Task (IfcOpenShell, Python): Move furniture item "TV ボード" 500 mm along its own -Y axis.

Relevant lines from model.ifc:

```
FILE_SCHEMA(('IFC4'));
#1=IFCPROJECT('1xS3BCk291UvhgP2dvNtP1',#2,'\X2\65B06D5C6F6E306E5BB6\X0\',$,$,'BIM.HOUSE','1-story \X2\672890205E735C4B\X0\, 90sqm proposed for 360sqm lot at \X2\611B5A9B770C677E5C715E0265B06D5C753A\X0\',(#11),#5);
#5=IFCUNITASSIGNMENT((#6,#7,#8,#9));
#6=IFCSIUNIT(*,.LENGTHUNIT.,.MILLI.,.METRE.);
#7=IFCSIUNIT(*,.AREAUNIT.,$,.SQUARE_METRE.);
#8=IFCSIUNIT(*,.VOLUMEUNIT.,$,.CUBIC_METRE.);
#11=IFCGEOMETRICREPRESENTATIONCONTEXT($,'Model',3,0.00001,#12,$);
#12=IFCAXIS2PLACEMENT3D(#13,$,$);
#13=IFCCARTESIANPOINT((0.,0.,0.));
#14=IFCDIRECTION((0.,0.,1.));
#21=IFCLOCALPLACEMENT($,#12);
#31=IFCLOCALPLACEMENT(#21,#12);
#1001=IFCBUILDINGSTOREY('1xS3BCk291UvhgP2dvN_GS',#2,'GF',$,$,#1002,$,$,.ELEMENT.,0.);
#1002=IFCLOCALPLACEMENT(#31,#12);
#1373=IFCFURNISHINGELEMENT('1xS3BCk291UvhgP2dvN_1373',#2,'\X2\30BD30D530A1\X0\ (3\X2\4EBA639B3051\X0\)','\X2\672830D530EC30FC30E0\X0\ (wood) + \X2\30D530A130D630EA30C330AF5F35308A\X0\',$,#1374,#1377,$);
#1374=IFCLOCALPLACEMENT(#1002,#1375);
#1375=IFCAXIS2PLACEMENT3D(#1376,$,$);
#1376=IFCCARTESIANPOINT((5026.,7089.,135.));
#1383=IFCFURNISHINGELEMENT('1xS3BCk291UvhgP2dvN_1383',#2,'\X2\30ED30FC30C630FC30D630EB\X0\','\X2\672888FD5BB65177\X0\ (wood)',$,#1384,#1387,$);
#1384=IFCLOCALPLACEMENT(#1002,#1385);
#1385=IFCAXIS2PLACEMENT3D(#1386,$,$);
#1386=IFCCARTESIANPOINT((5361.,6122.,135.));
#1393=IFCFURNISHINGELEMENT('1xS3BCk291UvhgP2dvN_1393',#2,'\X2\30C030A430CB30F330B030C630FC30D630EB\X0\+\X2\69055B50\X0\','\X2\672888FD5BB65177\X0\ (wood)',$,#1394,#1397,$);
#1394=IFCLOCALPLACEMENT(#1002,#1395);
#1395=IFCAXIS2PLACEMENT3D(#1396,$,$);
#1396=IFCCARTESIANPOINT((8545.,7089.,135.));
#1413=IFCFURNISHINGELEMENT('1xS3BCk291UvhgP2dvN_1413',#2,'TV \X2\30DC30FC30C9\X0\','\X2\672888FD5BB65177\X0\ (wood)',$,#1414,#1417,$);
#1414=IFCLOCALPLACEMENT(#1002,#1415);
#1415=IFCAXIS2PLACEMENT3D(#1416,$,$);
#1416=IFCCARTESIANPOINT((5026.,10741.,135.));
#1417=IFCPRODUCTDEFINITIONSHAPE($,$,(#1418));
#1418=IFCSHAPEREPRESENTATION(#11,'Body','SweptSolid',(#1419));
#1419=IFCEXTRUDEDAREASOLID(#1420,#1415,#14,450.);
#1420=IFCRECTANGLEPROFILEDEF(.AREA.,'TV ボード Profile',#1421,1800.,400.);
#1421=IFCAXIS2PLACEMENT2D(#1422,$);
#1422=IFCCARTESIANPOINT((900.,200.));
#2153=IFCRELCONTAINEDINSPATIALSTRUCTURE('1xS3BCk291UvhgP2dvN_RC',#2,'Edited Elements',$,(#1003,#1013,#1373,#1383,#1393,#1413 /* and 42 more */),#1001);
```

```python
import ifcopenshell
import ifcopenshell.api.geometry
import ifcopenshell.util.placement
import ifcopenshell.util.unit

model = ifcopenshell.open("model.ifc")
unit_scale = ifcopenshell.util.unit.calculate_unit_scale(model)

item = model.by_guid("1xS3BCk291UvhgP2dvN_1413")
matrix = ifcopenshell.util.placement.get_local_placement(item.ObjectPlacement)
matrix[:3, 3] -= matrix[:3, 1] * 0.5 / unit_scale
ifcopenshell.api.geometry.edit_object_placement(model, product=item, matrix=matrix, is_si=False)

print(ifcopenshell.util.placement.get_local_placement(item.ObjectPlacement).round(3) + 0.0)

model.write("model_v2.ifc")
```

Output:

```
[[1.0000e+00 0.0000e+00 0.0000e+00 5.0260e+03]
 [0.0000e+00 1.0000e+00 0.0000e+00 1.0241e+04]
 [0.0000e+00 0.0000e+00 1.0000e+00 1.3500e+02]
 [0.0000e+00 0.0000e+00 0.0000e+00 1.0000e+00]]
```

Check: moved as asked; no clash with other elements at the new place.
